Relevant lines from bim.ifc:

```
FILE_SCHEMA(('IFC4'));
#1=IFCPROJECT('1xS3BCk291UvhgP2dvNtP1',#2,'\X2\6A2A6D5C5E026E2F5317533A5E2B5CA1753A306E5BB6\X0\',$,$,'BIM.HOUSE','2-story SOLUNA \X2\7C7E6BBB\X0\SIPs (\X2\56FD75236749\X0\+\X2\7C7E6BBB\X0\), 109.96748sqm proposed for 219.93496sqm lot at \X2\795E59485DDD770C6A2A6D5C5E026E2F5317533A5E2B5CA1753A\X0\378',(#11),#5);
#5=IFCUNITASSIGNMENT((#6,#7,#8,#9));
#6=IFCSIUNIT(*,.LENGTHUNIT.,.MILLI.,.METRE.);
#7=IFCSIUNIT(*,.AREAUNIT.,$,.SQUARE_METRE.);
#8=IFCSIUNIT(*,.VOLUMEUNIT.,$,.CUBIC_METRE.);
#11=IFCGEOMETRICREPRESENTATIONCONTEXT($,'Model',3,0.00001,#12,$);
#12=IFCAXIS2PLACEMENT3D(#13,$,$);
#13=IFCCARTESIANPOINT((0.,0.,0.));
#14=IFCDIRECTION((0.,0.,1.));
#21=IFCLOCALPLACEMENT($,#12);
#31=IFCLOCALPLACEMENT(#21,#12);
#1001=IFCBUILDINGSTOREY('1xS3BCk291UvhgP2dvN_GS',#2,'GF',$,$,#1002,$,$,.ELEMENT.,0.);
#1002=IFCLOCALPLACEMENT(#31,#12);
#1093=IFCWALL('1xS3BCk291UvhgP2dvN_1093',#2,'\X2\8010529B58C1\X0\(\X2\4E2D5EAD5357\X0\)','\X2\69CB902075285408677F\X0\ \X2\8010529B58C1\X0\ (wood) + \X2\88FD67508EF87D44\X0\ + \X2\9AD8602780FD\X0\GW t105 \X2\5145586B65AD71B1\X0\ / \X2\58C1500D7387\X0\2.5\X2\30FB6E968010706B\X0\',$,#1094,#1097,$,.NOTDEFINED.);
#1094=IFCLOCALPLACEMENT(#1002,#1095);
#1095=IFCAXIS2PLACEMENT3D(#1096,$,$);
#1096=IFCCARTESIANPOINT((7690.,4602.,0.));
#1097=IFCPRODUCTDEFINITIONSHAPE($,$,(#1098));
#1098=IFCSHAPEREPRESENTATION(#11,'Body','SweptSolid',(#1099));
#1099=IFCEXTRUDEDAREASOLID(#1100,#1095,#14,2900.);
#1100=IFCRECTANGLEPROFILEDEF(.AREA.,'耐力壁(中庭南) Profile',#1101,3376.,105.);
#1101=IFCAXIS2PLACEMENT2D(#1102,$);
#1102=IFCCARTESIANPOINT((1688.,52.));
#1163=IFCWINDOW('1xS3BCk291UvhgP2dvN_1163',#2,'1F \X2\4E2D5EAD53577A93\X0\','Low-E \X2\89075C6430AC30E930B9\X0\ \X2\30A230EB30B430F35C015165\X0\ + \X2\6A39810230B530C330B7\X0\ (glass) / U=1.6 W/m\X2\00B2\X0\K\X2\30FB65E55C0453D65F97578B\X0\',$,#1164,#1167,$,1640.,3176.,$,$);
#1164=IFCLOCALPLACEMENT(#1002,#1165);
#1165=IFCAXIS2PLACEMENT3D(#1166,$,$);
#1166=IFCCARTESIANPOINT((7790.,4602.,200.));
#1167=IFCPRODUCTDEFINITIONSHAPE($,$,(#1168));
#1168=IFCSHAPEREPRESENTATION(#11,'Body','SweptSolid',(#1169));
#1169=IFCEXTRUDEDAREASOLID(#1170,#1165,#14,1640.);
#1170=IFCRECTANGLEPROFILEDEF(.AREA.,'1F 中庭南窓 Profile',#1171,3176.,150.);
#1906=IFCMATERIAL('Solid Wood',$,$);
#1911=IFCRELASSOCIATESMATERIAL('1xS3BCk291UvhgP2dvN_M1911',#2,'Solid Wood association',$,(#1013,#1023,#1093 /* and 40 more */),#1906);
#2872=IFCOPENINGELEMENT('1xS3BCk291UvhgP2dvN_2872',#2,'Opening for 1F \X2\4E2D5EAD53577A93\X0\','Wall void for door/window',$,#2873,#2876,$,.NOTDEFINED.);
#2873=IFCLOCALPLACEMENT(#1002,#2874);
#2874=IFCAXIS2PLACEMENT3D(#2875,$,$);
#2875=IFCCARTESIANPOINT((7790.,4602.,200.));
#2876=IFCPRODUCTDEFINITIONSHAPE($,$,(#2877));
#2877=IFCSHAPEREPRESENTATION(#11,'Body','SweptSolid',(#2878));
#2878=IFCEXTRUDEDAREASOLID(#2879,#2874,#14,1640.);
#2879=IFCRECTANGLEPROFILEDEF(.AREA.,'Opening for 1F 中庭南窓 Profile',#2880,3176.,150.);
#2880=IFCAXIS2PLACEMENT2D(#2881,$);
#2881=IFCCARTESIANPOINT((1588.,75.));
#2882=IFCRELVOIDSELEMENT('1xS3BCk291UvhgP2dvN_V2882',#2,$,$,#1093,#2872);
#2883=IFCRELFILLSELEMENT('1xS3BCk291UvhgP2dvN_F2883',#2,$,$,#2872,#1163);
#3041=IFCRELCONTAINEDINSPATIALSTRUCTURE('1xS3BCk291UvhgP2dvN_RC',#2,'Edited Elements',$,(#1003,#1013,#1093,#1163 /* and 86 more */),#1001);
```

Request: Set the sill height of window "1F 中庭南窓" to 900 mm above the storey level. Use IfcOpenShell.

```python
import numpy as np
import ifcopenshell
import ifcopenshell.api.geometry
import ifcopenshell.geom
import ifcopenshell.util.element
import ifcopenshell.util.placement
import ifcopenshell.util.shape
import ifcopenshell.util.unit

model = ifcopenshell.open("bim.ifc")
unit_scale = ifcopenshell.util.unit.calculate_unit_scale(model)

window = model.by_guid("1xS3BCk291UvhgP2dvN_1163")
opening = window.FillsVoids[0].RelatingOpeningElement
storey = ifcopenshell.util.element.get_container(window, ifc_class="IfcBuildingStorey")
level = ifcopenshell.util.placement.get_local_placement(storey.ObjectPlacement)[2, 3]

# The opening's origin need not be at the sill, so measure its lowest point.
shape = ifcopenshell.geom.create_shape(ifcopenshell.geom.settings(), opening)
bottom = ifcopenshell.util.shape.get_shape_bottom_elevation(shape, shape.geometry) / unit_scale
dz = level + 0.9 / unit_scale - bottom

shift = np.array([0.0, 0.0, dz])
# The window is not placed relative to its opening, so move both.
for product in (opening, window):
    matrix = ifcopenshell.util.placement.get_local_placement(product.ObjectPlacement)
    matrix[:3, 3] += shift
    ifcopenshell.api.geometry.edit_object_placement(model, product=product, matrix=matrix, is_si=False)

print(f"moved by {dz * unit_scale:+.3f} m")

model.write("bim_v2.ifc")
```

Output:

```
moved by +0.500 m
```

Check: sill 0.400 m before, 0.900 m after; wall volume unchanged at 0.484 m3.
